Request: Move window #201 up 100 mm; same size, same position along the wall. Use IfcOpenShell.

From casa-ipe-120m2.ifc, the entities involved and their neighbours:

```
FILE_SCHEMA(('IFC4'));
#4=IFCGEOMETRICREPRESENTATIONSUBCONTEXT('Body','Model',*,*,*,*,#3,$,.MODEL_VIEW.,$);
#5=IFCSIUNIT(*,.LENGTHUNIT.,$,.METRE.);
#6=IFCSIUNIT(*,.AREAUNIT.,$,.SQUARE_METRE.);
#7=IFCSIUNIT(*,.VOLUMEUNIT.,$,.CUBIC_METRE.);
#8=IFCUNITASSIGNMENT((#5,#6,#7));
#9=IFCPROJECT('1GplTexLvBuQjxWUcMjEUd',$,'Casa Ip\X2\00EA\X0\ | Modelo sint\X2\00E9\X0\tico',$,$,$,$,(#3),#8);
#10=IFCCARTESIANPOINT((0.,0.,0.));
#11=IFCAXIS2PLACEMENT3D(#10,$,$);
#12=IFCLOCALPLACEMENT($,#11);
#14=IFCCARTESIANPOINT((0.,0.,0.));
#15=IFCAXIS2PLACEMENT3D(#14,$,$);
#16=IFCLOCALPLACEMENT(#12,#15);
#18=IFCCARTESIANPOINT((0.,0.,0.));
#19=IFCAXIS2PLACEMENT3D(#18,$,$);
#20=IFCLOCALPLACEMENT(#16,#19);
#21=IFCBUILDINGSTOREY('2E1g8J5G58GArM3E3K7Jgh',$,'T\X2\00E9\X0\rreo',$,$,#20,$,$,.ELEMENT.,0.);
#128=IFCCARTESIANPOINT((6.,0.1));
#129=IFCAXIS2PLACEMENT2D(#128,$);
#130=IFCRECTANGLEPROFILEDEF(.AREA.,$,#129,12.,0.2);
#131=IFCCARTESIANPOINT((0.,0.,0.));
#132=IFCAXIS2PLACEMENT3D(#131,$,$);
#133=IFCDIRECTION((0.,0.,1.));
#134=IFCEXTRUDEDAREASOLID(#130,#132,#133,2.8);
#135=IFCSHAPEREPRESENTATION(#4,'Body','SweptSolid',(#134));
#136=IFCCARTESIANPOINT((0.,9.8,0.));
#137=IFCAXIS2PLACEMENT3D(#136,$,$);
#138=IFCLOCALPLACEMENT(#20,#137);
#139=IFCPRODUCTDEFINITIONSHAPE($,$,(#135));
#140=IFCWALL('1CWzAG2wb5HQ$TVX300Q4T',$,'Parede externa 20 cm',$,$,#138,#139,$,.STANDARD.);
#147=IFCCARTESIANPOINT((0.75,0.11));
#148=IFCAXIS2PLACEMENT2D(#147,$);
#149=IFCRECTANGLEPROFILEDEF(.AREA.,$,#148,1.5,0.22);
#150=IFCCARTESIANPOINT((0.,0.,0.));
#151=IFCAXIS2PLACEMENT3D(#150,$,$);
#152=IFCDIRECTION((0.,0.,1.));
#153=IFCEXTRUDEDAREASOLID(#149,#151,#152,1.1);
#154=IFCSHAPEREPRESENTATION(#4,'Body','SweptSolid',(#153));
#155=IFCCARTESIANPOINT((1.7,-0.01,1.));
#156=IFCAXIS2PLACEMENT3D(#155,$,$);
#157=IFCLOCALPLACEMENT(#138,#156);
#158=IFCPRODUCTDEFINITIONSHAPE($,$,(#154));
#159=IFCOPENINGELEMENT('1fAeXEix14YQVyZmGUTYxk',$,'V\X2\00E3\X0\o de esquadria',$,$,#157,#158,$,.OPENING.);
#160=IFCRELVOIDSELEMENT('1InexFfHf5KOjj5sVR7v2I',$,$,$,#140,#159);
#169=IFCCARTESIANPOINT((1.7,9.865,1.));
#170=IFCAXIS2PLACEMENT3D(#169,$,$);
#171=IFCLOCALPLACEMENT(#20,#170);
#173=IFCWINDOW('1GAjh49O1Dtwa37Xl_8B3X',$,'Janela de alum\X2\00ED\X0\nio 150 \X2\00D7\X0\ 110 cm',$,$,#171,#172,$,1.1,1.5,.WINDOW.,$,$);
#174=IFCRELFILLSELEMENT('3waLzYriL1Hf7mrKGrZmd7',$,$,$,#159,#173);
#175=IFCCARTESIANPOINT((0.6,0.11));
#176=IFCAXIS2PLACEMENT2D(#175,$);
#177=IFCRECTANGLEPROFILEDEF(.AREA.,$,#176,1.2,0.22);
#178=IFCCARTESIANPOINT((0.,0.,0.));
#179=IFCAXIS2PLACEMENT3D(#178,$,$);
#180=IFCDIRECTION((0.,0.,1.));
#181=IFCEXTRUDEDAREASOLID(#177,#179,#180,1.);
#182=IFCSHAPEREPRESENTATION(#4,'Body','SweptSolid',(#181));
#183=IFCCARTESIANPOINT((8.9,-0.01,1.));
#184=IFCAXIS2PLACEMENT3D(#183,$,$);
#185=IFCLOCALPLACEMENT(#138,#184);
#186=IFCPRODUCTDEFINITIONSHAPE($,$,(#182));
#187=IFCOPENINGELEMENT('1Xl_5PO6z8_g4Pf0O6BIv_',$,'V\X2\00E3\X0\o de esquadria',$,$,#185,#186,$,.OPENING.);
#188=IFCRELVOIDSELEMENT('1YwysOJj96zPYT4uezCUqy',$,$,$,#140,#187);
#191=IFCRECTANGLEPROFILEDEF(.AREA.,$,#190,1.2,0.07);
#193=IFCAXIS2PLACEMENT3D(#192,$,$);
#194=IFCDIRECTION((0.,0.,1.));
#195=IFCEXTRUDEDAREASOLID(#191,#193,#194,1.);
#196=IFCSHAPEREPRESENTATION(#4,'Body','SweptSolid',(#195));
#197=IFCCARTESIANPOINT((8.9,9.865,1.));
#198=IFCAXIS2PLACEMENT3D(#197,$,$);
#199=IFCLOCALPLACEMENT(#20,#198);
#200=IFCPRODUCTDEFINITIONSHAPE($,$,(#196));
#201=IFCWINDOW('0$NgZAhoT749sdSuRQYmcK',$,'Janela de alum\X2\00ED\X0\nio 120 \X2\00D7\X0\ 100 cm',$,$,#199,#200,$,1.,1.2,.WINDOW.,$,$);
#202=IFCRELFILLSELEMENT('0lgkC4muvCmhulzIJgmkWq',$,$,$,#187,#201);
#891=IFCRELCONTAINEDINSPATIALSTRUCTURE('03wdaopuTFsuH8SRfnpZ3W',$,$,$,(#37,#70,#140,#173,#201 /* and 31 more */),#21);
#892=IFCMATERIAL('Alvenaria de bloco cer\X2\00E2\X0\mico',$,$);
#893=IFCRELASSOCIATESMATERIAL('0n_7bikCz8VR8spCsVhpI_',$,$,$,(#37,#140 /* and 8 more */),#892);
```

```python
import numpy as np
import ifcopenshell
import ifcopenshell.api.geometry
import ifcopenshell.util.placement
import ifcopenshell.util.unit

model = ifcopenshell.open("casa-ipe-120m2.ifc")
unit_scale = ifcopenshell.util.unit.calculate_unit_scale(model)

window = model.by_guid("0$NgZAhoT749sdSuRQYmcK")
opening = window.FillsVoids[0].RelatingOpeningElement
dz = 0.1 / unit_scale

shift = np.array([0.0, 0.0, dz])
# The window is not placed relative to its opening, so move both.
for product in (opening, window):
    matrix = ifcopenshell.util.placement.get_local_placement(product.ObjectPlacement)
    matrix[:3, 3] += shift
    ifcopenshell.api.geometry.edit_object_placement(model, product=product, matrix=matrix, is_si=False)

print(f"moved by {dz * unit_scale:+.3f} m")

model.write("casa-ipe-120m2_updated.ifc")
```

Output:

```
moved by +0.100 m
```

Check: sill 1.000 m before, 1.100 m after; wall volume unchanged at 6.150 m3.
